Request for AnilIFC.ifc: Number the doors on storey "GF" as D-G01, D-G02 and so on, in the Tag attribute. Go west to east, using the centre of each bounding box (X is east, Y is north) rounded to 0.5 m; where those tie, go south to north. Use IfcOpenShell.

First a look at what the model holds.

```python
import ifcopenshell
import ifcopenshell.util.element
import ifcopenshell.util.placement

model = ifcopenshell.open("AnilIFC.ifc")
print(model.schema)
storey = next(s for s in model.by_type("IfcBuildingStorey") if s.Name == "GF")
doors = [e for e in ifcopenshell.util.element.get_decomposition(storey) if e.is_a("IfcDoor")]
for e in sorted(doors, key=lambda e: e.id()):
    origin = ifcopenshell.util.placement.get_local_placement(e.ObjectPlacement)[:3, 3]
    print(e.id(), e.Tag, e.Name, origin.round(2) + 0.0, sep=" | ")
```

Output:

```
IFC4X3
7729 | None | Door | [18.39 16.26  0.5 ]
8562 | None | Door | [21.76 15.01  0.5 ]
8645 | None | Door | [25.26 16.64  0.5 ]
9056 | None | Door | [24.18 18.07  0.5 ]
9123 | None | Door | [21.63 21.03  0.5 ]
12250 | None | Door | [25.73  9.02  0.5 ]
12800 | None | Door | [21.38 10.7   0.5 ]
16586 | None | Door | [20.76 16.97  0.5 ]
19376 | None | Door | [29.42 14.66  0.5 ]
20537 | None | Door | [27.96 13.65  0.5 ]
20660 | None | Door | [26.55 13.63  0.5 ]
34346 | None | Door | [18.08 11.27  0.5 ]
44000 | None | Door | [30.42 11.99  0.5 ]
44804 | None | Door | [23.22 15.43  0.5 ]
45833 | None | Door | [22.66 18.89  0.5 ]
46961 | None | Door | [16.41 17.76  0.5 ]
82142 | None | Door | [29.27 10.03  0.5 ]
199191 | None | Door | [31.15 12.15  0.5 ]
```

```python
import ifcopenshell
import ifcopenshell.geom
import ifcopenshell.util.element
import ifcopenshell.util.shape

model = ifcopenshell.open("AnilIFC.ifc")
settings = ifcopenshell.geom.settings()
settings.set("use-world-coords", True)


def centre(element):
    shape = ifcopenshell.geom.create_shape(settings, element)
    return ifcopenshell.util.shape.get_bbox_centroid(shape.geometry)


storey = next(s for s in model.by_type("IfcBuildingStorey") if s.Name == "GF")
doors = [e for e in ifcopenshell.util.element.get_decomposition(storey) if e.is_a("IfcDoor")]

# Insertion points can sit at a corner or the storey origin, so sort by the geometry (in metres).
centres = {e: centre(e) for e in doors}
doors.sort(key=lambda e: (round(centres[e][0] / 0.5), centres[e][1]))

for i, e in enumerate(doors, start=1):
    number = f"D-G{i:02d}"
    e.Tag = number
    print(e.id(), number)

model.write("AnilIFC_updated.ifc")
```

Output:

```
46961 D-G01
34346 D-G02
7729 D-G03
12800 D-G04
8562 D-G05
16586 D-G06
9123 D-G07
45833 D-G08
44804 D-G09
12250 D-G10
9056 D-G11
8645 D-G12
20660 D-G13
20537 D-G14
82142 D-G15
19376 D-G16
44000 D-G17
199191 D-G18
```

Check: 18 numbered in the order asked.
